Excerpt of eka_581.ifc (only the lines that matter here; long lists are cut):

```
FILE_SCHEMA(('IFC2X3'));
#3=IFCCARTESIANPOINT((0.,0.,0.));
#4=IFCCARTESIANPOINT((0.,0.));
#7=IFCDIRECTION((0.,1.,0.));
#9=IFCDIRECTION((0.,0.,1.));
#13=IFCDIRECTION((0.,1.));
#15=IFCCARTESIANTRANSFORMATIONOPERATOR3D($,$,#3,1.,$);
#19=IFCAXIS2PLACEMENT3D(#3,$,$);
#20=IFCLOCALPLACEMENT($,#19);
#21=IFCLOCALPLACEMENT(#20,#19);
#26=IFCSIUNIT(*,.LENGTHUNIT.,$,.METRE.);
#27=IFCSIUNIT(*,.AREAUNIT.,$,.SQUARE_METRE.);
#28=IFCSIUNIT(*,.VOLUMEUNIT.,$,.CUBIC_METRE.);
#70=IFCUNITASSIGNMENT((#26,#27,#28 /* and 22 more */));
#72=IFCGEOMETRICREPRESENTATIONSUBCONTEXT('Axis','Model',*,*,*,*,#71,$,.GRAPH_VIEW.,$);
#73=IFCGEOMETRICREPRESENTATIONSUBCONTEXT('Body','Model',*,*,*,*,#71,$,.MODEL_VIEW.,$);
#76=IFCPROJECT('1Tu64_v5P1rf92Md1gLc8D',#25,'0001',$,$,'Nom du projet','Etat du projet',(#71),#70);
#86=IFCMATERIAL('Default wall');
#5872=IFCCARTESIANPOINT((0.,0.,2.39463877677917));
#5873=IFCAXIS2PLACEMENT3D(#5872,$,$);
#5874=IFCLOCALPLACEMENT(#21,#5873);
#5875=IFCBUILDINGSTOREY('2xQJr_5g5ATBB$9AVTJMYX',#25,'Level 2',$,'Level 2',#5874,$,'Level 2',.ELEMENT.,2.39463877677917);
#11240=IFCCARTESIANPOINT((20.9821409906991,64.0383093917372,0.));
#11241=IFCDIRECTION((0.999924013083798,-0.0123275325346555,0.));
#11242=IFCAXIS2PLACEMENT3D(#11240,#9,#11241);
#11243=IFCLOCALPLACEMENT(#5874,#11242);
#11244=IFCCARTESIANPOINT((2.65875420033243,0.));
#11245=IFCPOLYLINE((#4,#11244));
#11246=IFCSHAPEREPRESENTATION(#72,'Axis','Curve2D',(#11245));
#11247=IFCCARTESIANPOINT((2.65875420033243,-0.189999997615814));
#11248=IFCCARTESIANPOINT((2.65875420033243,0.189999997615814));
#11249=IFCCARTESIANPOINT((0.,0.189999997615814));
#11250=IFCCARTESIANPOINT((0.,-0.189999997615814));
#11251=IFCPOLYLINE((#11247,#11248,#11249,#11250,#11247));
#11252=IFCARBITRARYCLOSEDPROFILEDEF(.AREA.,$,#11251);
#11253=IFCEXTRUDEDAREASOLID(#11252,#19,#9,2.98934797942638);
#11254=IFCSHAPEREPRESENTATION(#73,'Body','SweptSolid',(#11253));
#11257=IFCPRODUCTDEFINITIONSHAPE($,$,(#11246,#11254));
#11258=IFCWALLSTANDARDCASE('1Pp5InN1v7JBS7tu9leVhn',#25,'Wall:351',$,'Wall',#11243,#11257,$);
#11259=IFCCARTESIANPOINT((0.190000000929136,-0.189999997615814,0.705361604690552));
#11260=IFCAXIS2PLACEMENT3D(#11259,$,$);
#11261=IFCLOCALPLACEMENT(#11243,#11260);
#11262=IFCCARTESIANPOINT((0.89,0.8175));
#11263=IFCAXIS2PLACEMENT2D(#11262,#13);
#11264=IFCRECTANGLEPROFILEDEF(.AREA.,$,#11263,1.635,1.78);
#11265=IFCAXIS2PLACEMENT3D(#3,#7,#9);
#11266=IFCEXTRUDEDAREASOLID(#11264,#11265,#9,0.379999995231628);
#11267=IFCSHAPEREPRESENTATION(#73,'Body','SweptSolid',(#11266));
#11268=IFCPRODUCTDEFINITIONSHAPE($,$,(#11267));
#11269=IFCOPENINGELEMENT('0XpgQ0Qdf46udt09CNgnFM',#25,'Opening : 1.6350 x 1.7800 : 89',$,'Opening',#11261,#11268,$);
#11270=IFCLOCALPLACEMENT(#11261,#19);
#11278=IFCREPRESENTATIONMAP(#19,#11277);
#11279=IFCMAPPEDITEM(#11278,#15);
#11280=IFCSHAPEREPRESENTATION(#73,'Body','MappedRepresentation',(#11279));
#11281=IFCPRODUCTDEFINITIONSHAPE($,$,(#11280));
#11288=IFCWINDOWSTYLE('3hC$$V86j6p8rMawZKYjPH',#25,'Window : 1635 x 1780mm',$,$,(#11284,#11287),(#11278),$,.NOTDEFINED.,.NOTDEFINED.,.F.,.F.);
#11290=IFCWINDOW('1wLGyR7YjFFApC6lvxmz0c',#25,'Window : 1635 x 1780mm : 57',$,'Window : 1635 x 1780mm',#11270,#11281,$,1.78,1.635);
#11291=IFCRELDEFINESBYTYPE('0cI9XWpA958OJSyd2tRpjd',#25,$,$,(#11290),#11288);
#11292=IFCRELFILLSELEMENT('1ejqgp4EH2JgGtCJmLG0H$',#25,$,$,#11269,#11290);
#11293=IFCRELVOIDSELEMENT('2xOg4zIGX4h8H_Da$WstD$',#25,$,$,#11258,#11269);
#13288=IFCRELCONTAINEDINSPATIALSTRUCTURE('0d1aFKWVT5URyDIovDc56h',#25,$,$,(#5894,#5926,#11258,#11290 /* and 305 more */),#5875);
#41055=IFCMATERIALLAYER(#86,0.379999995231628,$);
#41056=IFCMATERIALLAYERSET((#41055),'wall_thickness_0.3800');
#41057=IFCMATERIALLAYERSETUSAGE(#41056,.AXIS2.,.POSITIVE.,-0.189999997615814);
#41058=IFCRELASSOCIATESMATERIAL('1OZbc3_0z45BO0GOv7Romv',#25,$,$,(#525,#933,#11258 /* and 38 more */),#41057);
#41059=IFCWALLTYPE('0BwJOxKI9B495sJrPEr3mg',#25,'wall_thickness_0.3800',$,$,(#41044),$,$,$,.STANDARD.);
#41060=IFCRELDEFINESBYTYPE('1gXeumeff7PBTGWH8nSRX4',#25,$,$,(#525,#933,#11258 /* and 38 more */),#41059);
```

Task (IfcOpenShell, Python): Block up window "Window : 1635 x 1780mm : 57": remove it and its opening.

```python
import ifcopenshell
import ifcopenshell.api.feature
import ifcopenshell.api.root
import ifcopenshell.geom
import ifcopenshell.util.shape

model = ifcopenshell.open("eka_581.ifc")
settings = ifcopenshell.geom.settings()


def volume(element):
    """Net volume in cubic metres, openings subtracted."""
    shape = ifcopenshell.geom.create_shape(settings, element)
    return ifcopenshell.util.shape.get_volume(shape.geometry)


window = model.by_guid("1wLGyR7YjFFApC6lvxmz0c")
opening = window.FillsVoids[0].RelatingOpeningElement
wall = opening.VoidsElements[0].RelatingBuildingElement
before = volume(wall)

ifcopenshell.api.root.remove_product(model, product=window)
ifcopenshell.api.feature.remove_feature(model, feature=opening)

after = volume(wall)

print(f"wall volume {before:.3f} -> {after:.3f} m3")

model.write("eka_581_updated.ifc")
```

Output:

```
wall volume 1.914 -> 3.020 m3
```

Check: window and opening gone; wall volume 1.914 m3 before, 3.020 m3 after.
